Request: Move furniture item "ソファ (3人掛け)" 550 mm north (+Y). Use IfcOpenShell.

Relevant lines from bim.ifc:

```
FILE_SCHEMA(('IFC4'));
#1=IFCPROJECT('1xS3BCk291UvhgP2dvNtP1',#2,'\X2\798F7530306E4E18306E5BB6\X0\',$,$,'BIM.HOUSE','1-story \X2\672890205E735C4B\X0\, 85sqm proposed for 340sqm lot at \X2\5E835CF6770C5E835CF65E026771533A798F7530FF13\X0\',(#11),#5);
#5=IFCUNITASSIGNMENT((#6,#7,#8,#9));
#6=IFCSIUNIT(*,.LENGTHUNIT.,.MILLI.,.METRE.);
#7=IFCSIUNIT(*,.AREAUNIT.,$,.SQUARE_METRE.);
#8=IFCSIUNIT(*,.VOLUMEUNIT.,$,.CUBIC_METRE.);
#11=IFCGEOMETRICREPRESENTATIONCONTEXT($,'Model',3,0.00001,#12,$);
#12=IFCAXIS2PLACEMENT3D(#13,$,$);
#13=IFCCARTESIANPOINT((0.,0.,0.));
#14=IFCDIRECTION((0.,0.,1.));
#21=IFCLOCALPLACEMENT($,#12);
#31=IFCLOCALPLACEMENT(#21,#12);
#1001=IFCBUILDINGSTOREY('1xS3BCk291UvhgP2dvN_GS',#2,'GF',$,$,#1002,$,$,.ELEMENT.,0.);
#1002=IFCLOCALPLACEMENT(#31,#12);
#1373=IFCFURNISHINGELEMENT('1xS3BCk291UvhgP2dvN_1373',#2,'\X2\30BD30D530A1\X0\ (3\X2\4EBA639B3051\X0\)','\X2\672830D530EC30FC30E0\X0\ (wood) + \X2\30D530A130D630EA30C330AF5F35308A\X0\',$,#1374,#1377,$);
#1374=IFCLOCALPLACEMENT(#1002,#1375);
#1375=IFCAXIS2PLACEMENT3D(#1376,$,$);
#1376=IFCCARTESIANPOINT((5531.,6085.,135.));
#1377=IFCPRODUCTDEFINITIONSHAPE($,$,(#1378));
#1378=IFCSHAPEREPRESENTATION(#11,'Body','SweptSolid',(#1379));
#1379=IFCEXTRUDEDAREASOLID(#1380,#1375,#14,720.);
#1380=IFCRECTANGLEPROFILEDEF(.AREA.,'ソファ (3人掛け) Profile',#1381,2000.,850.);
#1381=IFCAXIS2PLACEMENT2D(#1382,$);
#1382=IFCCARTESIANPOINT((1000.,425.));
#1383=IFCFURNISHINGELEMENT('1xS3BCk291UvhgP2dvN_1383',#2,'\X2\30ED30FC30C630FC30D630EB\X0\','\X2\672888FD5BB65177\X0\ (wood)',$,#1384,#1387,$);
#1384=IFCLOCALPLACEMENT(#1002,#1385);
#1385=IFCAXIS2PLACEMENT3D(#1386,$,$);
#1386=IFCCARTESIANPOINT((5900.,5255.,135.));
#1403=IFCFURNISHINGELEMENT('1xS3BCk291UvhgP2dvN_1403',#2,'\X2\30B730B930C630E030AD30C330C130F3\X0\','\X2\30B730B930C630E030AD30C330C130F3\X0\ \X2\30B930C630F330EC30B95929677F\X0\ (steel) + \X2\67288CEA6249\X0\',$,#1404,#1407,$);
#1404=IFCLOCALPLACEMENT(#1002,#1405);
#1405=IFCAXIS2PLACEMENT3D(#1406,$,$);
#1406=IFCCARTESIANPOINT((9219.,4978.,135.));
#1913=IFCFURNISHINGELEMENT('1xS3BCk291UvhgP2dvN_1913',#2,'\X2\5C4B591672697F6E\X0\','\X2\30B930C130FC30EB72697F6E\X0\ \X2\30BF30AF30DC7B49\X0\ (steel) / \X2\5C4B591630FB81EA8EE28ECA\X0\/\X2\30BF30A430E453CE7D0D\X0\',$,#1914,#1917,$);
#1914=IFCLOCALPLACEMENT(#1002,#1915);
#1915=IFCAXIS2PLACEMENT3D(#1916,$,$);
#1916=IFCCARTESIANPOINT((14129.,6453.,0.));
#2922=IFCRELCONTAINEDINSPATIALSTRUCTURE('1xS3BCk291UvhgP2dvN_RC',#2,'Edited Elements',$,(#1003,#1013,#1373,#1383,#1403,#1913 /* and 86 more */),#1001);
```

```python
import ifcopenshell
import ifcopenshell.api.geometry
import ifcopenshell.util.placement
import ifcopenshell.util.unit

model = ifcopenshell.open("bim.ifc")
unit_scale = ifcopenshell.util.unit.calculate_unit_scale(model)

item = model.by_guid("1xS3BCk291UvhgP2dvN_1373")
matrix = ifcopenshell.util.placement.get_local_placement(item.ObjectPlacement)
matrix[1, 3] += 0.55 / unit_scale
ifcopenshell.api.geometry.edit_object_placement(model, product=item, matrix=matrix, is_si=False)

print(ifcopenshell.util.placement.get_local_placement(item.ObjectPlacement).round(3) + 0.0)

model.write("bim_rev.ifc")
```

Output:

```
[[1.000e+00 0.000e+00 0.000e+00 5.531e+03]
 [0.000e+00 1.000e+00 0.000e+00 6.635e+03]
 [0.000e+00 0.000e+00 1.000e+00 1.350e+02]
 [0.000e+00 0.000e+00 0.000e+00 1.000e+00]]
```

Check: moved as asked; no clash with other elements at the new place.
